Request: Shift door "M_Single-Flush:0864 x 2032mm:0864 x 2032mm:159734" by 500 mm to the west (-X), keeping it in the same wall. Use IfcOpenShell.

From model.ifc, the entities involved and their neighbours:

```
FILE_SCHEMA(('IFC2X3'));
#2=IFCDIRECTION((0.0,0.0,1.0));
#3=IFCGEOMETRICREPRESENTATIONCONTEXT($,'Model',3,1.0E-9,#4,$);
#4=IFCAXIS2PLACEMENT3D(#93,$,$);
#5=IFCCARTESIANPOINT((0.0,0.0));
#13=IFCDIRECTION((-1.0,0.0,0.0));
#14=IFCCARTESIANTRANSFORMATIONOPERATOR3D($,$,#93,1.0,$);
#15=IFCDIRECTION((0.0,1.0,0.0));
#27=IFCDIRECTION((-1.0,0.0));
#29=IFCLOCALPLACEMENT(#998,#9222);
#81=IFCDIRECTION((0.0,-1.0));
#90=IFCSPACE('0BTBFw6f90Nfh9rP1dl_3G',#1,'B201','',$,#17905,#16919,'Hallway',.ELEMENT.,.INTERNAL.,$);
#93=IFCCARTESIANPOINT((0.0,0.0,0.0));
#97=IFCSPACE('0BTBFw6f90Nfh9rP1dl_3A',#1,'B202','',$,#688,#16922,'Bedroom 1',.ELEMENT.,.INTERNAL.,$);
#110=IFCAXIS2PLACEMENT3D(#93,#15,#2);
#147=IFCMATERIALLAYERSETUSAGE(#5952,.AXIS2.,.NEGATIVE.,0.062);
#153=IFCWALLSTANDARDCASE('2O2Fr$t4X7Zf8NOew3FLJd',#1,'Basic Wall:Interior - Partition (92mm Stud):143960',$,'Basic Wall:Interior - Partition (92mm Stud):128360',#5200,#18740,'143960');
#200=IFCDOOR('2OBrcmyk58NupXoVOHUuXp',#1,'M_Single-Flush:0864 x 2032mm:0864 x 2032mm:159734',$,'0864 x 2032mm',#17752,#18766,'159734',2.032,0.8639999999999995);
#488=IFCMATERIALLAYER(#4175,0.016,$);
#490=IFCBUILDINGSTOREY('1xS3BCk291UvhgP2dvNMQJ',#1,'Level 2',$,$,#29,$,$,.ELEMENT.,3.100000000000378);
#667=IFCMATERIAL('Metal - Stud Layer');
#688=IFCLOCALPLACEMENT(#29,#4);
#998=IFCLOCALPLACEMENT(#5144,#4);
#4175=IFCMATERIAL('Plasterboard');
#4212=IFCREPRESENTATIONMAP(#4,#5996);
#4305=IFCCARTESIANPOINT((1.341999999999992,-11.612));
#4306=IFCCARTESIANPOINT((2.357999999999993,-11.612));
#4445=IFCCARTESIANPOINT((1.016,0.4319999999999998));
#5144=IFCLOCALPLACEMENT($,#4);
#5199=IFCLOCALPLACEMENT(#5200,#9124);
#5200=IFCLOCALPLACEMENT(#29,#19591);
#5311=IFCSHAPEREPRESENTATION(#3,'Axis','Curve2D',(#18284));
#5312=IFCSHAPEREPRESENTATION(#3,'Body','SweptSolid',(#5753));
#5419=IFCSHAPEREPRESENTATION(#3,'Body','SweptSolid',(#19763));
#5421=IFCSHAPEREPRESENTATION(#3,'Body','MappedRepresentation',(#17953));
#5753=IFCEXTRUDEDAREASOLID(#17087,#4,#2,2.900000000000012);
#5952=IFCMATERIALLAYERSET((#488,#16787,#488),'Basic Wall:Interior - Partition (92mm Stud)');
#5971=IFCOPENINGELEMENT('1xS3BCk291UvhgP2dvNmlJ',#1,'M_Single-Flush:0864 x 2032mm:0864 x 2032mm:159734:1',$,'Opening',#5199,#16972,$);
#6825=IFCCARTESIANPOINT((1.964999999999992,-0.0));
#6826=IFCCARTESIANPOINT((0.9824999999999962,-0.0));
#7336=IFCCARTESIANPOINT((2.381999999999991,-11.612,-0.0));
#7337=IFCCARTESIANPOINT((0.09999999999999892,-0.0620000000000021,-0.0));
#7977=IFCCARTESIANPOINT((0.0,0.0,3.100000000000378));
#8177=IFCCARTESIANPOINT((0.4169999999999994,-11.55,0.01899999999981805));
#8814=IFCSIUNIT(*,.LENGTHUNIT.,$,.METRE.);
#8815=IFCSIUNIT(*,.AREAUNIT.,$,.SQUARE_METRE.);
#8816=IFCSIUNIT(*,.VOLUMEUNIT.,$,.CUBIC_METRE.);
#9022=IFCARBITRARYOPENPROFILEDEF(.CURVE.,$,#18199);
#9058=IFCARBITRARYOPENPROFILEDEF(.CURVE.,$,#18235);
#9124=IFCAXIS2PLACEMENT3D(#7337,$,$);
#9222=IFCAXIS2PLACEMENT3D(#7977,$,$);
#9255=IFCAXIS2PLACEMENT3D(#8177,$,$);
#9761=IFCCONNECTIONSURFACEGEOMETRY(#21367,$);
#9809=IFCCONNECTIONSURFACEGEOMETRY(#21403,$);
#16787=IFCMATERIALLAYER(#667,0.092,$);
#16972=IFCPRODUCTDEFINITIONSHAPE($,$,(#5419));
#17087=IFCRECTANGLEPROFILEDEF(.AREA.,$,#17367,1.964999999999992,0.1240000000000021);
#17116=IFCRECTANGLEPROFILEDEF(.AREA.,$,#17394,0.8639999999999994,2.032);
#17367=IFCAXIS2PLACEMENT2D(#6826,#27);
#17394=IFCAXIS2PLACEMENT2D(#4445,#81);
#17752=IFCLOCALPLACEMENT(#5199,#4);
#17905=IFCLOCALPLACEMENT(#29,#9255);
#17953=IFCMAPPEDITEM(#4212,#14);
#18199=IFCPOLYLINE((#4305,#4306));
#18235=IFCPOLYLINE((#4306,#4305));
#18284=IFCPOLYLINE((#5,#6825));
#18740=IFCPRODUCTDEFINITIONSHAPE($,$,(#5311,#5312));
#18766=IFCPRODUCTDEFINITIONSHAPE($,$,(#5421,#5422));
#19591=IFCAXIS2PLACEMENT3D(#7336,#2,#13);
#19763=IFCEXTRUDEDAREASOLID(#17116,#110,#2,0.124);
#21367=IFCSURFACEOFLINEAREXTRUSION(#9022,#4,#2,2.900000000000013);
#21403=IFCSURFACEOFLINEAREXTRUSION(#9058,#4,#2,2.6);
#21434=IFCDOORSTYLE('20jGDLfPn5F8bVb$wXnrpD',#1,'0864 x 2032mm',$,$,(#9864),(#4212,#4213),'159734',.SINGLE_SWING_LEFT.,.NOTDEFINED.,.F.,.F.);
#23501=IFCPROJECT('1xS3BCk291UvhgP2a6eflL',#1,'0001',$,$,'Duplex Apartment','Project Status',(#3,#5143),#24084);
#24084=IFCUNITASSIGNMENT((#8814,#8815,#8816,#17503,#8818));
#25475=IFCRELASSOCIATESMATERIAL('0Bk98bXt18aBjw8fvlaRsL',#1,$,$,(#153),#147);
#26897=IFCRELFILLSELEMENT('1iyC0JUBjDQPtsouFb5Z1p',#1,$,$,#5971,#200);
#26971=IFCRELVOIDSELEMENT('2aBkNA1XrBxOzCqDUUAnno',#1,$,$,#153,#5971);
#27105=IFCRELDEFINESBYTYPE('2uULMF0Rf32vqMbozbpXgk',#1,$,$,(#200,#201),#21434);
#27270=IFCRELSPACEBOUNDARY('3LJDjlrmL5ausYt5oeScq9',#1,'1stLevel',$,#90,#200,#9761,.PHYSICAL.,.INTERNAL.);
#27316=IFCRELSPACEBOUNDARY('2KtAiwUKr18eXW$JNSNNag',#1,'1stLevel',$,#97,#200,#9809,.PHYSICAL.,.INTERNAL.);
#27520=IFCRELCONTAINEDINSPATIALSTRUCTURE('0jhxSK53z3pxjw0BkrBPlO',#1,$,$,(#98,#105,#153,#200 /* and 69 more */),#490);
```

```python
import numpy as np
import ifcopenshell
import ifcopenshell.api.geometry
import ifcopenshell.util.placement

model = ifcopenshell.open("model.ifc")

door = model.by_guid("2OBrcmyk58NupXoVOHUuXp")
opening = door.FillsVoids[0].RelatingOpeningElement
wall = opening.VoidsElements[0].RelatingBuildingElement

wall_matrix = ifcopenshell.util.placement.get_local_placement(wall.ObjectPlacement)
shift = wall_matrix[:3, 0] * 0.5
before = ifcopenshell.util.placement.get_local_placement(door.ObjectPlacement)[:3, 3].copy()

# The door is placed relative to its opening, so it follows when the opening moves.
matrix = ifcopenshell.util.placement.get_local_placement(opening.ObjectPlacement)
matrix[:3, 3] += shift
ifcopenshell.api.geometry.edit_object_placement(
    model, product=opening, matrix=matrix, is_si=False, should_transform_children=True
)

# Space boundary surfaces are stored in each space's coordinates; move them too.
for rel in door.ProvidesBoundaries:
    if not rel.ConnectionGeometry:
        continue
    surface = rel.ConnectionGeometry.SurfaceOnRelatingElement
    space_matrix = ifcopenshell.util.placement.get_local_placement(rel.RelatingSpace.ObjectPlacement)
    point = np.array(surface.Position.Location.Coordinates) + space_matrix[:3, :3].T @ shift
    surface.Position = model.createIfcAxis2Placement3D(
        model.createIfcCartesianPoint(point.tolist()), surface.Position.Axis, surface.Position.RefDirection
    )

after = ifcopenshell.util.placement.get_local_placement(door.ObjectPlacement)[:3, 3]
print("door moved by", (after - before).round(3) + 0.0)

model.write("model_rev.ifc")
```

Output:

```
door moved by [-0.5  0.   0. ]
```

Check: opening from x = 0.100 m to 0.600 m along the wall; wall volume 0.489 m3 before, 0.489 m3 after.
